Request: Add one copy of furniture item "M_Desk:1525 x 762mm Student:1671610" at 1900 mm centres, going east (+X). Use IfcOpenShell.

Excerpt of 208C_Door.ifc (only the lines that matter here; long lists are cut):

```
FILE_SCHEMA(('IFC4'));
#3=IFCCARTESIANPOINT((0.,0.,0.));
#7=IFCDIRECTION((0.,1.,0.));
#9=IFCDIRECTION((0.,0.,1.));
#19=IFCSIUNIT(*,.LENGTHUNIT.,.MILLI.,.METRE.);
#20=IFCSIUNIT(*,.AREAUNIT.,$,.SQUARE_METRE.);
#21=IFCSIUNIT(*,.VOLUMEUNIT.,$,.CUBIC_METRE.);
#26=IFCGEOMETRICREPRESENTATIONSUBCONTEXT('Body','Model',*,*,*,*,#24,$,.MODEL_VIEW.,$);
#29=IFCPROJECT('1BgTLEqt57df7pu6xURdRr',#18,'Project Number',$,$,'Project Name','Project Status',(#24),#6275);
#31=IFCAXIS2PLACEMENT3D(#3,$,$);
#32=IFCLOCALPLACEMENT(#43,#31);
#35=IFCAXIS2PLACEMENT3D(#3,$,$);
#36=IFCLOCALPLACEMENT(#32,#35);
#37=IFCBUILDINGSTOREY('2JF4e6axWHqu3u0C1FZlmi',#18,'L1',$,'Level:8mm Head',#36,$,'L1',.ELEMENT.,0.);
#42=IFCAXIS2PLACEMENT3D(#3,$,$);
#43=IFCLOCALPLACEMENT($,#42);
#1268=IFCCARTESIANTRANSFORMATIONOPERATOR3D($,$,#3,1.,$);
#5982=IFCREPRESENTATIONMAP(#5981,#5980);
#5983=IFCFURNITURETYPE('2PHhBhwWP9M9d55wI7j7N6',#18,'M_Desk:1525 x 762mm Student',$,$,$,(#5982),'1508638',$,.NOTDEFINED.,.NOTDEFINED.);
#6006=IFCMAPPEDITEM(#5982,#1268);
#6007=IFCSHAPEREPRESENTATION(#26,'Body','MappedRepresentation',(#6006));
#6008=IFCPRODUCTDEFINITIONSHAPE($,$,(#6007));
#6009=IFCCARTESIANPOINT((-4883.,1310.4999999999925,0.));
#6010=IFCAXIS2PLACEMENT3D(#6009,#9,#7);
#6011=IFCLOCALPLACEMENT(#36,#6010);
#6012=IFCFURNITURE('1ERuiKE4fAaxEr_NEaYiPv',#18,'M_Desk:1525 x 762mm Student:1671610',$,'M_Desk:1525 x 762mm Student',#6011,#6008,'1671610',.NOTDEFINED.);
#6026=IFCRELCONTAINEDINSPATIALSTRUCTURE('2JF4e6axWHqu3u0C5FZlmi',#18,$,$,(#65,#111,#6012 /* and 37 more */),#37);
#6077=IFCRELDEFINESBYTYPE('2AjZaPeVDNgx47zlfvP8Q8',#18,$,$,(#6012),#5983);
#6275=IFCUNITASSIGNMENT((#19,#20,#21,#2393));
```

```python
import numpy as np
import ifcopenshell
import ifcopenshell.api.geometry
import ifcopenshell.api.root
import ifcopenshell.util.element
import ifcopenshell.util.placement

model = ifcopenshell.open("208C_Door.ifc")


def reuse_history(source, copy):
    """copy_class also copies each property set's owner history, people and application; keep the originals."""
    for rel in copy.IsDefinedBy:
        if rel.is_a("IfcRelDefinesByProperties") and (history := rel.RelatingPropertyDefinition.OwnerHistory):
            rel.RelatingPropertyDefinition.OwnerHistory = source.OwnerHistory
            ifcopenshell.util.element.remove_deep2(model, history)


source = model.by_guid("1ERuiKE4fAaxEr_NEaYiPv")
base = ifcopenshell.util.placement.get_local_placement(source.ObjectPlacement)
step = np.array([1.0, 0.0, 0.0]) * 1900.0

for i in range(1, 2):
    copy = ifcopenshell.api.root.copy_class(model, product=source)
    copy.Representation = ifcopenshell.util.element.copy_deep(
        model, source.Representation, exclude=["IfcGeometricRepresentationContext", "IfcRepresentationMap"]
    )
    copy.Name = "M_Desk:1525 x 762mm Student"
    copy.Tag = None
    reuse_history(source, copy)
    matrix = base.copy()
    matrix[:3, 3] += i * step
    print("added at", matrix[:3, 3].round(3) + 0.0)
    ifcopenshell.api.geometry.edit_object_placement(model, product=copy, matrix=matrix, is_si=False)

model.write("208C_Door_edited.ifc")
```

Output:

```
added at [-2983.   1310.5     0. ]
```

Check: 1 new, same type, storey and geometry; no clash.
